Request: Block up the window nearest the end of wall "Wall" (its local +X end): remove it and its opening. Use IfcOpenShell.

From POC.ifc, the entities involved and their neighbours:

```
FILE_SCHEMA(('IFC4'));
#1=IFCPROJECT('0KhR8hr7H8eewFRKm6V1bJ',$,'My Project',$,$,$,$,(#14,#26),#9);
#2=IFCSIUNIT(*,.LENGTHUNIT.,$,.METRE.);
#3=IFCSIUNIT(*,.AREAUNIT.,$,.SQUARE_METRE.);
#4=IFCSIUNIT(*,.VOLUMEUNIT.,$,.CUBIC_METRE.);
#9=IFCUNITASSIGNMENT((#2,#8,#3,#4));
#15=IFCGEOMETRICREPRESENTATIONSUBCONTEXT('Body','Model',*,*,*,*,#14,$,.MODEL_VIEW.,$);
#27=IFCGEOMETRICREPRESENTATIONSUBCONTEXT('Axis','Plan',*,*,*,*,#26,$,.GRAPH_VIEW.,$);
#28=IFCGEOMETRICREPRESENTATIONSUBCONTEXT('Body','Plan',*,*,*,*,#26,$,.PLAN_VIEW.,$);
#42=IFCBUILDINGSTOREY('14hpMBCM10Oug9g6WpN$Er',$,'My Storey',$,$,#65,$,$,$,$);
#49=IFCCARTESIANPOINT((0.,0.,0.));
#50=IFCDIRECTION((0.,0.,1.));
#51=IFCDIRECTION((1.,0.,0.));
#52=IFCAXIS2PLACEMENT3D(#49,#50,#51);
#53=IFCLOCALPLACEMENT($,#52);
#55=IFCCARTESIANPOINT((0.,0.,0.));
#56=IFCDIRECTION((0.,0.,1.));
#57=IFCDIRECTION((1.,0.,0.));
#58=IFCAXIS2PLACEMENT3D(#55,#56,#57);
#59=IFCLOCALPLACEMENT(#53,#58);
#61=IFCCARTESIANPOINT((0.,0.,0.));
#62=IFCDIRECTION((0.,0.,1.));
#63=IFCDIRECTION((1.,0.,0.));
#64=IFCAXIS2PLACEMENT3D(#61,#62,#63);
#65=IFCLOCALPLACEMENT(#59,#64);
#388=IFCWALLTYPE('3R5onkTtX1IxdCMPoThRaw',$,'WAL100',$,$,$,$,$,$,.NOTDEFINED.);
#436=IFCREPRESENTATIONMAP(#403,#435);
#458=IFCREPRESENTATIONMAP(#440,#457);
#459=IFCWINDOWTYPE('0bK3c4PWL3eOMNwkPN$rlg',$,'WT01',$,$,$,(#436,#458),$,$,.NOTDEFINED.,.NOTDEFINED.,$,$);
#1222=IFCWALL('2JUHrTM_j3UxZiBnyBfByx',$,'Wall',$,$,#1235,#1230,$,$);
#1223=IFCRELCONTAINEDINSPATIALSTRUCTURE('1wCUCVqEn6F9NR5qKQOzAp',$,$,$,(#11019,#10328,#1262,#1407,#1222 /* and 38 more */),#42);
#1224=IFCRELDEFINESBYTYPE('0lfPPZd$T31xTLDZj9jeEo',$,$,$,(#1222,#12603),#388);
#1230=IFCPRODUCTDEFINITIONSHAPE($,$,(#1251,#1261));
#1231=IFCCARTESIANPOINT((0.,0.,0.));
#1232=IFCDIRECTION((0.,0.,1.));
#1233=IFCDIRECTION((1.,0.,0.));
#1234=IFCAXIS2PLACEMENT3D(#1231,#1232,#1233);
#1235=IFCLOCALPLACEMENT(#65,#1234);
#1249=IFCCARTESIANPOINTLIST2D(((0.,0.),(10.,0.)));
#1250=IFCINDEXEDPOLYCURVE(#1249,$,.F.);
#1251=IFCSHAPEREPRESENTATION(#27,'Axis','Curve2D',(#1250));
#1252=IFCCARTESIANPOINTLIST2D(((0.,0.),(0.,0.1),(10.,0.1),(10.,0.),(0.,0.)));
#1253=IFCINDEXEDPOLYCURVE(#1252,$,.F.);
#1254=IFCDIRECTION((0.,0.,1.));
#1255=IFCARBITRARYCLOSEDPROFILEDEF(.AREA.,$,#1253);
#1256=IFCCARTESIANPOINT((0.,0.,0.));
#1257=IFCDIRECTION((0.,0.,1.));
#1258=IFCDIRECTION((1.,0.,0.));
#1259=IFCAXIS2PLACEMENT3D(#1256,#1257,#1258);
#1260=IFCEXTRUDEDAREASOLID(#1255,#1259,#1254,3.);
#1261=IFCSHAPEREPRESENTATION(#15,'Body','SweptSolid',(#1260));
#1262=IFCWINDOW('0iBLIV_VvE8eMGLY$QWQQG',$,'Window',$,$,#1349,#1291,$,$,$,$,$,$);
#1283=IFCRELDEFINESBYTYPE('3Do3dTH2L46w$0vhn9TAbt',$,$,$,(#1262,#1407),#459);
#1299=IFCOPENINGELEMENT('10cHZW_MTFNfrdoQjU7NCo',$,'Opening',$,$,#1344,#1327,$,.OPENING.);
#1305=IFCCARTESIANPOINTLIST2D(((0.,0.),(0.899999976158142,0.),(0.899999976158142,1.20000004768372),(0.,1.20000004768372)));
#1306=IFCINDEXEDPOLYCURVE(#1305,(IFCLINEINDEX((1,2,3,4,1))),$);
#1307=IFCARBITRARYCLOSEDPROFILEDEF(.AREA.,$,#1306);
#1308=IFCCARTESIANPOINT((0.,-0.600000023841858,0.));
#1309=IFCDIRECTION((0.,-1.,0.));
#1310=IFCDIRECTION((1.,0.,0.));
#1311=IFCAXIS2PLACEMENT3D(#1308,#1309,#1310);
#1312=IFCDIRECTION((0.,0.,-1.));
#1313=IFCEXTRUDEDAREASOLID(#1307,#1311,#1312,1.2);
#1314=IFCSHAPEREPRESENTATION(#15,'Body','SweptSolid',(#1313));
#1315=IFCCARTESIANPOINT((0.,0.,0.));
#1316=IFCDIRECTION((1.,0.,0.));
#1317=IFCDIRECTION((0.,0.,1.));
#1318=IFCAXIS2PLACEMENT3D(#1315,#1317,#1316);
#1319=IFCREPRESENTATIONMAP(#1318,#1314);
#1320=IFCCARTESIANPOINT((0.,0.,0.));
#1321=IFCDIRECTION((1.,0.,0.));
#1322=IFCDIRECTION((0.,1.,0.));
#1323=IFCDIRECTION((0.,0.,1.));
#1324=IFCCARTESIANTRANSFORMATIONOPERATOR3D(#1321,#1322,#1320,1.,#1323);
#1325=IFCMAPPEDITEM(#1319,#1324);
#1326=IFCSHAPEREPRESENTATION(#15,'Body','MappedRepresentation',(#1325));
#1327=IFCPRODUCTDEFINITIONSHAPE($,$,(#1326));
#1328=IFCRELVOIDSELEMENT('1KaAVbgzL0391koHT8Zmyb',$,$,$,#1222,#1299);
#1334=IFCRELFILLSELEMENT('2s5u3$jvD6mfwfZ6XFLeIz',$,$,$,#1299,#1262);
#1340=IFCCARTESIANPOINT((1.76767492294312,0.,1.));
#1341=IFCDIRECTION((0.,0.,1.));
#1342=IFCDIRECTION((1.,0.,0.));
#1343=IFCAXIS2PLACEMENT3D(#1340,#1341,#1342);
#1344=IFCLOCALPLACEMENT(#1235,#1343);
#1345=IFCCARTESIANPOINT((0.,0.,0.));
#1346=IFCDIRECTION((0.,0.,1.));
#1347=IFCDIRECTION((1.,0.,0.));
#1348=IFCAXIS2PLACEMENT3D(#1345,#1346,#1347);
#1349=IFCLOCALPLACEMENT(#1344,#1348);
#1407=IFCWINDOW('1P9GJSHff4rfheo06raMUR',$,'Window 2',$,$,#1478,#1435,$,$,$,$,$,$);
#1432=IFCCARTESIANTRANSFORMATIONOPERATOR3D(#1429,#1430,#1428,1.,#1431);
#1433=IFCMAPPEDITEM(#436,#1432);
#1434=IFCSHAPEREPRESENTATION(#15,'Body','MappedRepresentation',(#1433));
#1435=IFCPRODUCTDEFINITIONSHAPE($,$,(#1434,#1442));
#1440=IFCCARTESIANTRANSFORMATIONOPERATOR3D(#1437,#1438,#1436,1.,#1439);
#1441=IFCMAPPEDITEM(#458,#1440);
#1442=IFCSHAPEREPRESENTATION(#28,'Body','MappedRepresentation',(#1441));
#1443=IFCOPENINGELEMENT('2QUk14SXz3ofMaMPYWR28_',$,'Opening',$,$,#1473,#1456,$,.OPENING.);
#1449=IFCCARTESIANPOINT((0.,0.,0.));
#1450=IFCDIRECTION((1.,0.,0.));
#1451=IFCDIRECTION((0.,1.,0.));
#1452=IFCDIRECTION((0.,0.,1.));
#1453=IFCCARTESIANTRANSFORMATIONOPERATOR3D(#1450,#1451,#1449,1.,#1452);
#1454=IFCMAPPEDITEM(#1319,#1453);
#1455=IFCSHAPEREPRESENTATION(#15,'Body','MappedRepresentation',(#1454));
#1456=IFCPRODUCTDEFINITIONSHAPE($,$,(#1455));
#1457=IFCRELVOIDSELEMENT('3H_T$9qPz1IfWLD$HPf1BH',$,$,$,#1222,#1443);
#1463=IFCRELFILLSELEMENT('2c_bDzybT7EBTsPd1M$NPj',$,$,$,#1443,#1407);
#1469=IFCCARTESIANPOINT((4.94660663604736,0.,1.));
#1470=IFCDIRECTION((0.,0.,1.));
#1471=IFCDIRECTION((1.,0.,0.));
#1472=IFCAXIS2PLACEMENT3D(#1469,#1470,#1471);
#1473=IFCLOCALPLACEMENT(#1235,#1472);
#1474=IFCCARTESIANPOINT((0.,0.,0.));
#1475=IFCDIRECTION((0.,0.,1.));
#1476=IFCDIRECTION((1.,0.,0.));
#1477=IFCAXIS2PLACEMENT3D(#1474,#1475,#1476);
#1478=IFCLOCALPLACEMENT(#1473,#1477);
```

```python
import ifcopenshell
import ifcopenshell.api.feature
import ifcopenshell.api.root
import ifcopenshell.geom
import ifcopenshell.util.shape

model = ifcopenshell.open("POC.ifc")
settings = ifcopenshell.geom.settings()


def volume(element):
    """Net volume in cubic metres, openings subtracted."""
    shape = ifcopenshell.geom.create_shape(settings, element)
    return ifcopenshell.util.shape.get_volume(shape.geometry)


window = model.by_guid("1P9GJSHff4rfheo06raMUR")
opening = window.FillsVoids[0].RelatingOpeningElement
wall = opening.VoidsElements[0].RelatingBuildingElement
before = volume(wall)

ifcopenshell.api.root.remove_product(model, product=window)
ifcopenshell.api.feature.remove_feature(model, feature=opening)

after = volume(wall)

print(f"wall volume {before:.3f} -> {after:.3f} m3")

model.write("POC_v2.ifc")
```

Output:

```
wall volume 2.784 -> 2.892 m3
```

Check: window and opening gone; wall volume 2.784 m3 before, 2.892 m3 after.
